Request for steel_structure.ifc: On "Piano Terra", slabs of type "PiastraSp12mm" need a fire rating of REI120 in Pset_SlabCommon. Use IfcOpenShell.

First a look at what the model holds.

```python
import ifcopenshell
import ifcopenshell.util.element

model = ifcopenshell.open("steel_structure.ifc")
print(model.schema)
storey = next(s for s in model.by_type("IfcBuildingStorey") if s.Name == "Piano Terra")
slabs = [e for e in ifcopenshell.util.element.get_decomposition(storey) if e.is_a("IfcSlab")]
seen = {}
for e in slabs:
    element_type = ifcopenshell.util.element.get_type(e)
    key = (element_type.Name if element_type != e and element_type else None, ifcopenshell.util.element.get_pset(e, "Pset_SlabCommon", "FireRating"))
    seen[key] = seen.get(key, 0) + 1
for (name, value), count in sorted(seen.items(), key=str):
    print(count, "x", name, "|", value)
```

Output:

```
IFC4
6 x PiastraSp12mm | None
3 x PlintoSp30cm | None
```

```python
import ifcopenshell
import ifcopenshell.api.pset
import ifcopenshell.util.element

model = ifcopenshell.open("steel_structure.ifc")

storey = next(s for s in model.by_type("IfcBuildingStorey") if s.Name == "Piano Terra")
slabs = [e for e in ifcopenshell.util.element.get_decomposition(storey) if e.is_a("IfcSlab")]

count = 0
for e in slabs:
    element_type = ifcopenshell.util.element.get_type(e)
    if element_type in (None, e) or element_type.Name != "PiastraSp12mm":
        continue
    # add_pset returns the element's existing set when there is one.
    pset = ifcopenshell.api.pset.add_pset(model, product=e, name="Pset_SlabCommon")
    ifcopenshell.api.pset.edit_pset(model, pset=pset, properties={"FireRating": "REI120"})
    count += 1

print(count, "slabs updated")

model.write("steel_structure_edited.ifc")
```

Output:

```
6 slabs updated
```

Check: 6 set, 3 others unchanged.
